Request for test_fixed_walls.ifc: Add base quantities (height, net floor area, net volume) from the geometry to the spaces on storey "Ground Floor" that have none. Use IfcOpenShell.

First a look at what the model holds.

```python
import ifcopenshell
import ifcopenshell.util.element
import ifcopenshell.util.unit

model = ifcopenshell.open("test_fixed_walls.ifc")
print(model.schema)
for unit_type in ("LENGTHUNIT", "AREAUNIT", "VOLUMEUNIT"):
    print(unit_type, ifcopenshell.util.unit.calculate_unit_scale(model, unit_type))
storey = next(s for s in model.by_type("IfcBuildingStorey") if s.Name == "Ground Floor")
spaces = [e for e in ifcopenshell.util.element.get_decomposition(storey) if e.is_a("IfcSpace")]
for e in sorted(spaces, key=lambda e: e.id()):
    print(e.id(), e.is_a(), e.Name, list(ifcopenshell.util.element.get_psets(e, qtos_only=True)), sep=" | ")
```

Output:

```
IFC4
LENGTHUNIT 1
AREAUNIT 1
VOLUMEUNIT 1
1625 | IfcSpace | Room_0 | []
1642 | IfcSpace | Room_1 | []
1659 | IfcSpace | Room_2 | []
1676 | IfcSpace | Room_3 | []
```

```python
import ifcopenshell
import ifcopenshell.api.pset
import ifcopenshell.geom
import ifcopenshell.util.element
import ifcopenshell.util.shape
import ifcopenshell.util.unit

model = ifcopenshell.open("test_fixed_walls.ifc")
unit_scale = ifcopenshell.util.unit.calculate_unit_scale(model)
area_scale = ifcopenshell.util.unit.calculate_unit_scale(model, "AREAUNIT")
volume_scale = ifcopenshell.util.unit.calculate_unit_scale(model, "VOLUMEUNIT")
settings = ifcopenshell.geom.settings()

storey = next(s for s in model.by_type("IfcBuildingStorey") if s.Name == "Ground Floor")
spaces = [e for e in ifcopenshell.util.element.get_decomposition(storey) if e.is_a("IfcSpace")]

for e in sorted(spaces, key=lambda e: e.id()):
    if ifcopenshell.util.element.get_psets(e, qtos_only=True, should_inherit=False):
        continue
    # Geometry comes back in metres, in the element's own axes.
    shape = ifcopenshell.geom.create_shape(settings, e)
    values = {
        "Height": ifcopenshell.util.shape.get_z(shape.geometry) / unit_scale,
        "NetFloorArea": ifcopenshell.util.shape.get_footprint_area(shape.geometry) / area_scale,
        "NetVolume": ifcopenshell.util.shape.get_volume(shape.geometry) / volume_scale,
    }
    qto = ifcopenshell.api.pset.add_qto(model, product=e, name="Qto_SpaceBaseQuantities")
    ifcopenshell.api.pset.edit_qto(model, qto=qto, properties=values)
    print(e.id(), {k: round(v, 3) for k, v in values.items()})

model.write("test_fixed_walls_rev.ifc")
```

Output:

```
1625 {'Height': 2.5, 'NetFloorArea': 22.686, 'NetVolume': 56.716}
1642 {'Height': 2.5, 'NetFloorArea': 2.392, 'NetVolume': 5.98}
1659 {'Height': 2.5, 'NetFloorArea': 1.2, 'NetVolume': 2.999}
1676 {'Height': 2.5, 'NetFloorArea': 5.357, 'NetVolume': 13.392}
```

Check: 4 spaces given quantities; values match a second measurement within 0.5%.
